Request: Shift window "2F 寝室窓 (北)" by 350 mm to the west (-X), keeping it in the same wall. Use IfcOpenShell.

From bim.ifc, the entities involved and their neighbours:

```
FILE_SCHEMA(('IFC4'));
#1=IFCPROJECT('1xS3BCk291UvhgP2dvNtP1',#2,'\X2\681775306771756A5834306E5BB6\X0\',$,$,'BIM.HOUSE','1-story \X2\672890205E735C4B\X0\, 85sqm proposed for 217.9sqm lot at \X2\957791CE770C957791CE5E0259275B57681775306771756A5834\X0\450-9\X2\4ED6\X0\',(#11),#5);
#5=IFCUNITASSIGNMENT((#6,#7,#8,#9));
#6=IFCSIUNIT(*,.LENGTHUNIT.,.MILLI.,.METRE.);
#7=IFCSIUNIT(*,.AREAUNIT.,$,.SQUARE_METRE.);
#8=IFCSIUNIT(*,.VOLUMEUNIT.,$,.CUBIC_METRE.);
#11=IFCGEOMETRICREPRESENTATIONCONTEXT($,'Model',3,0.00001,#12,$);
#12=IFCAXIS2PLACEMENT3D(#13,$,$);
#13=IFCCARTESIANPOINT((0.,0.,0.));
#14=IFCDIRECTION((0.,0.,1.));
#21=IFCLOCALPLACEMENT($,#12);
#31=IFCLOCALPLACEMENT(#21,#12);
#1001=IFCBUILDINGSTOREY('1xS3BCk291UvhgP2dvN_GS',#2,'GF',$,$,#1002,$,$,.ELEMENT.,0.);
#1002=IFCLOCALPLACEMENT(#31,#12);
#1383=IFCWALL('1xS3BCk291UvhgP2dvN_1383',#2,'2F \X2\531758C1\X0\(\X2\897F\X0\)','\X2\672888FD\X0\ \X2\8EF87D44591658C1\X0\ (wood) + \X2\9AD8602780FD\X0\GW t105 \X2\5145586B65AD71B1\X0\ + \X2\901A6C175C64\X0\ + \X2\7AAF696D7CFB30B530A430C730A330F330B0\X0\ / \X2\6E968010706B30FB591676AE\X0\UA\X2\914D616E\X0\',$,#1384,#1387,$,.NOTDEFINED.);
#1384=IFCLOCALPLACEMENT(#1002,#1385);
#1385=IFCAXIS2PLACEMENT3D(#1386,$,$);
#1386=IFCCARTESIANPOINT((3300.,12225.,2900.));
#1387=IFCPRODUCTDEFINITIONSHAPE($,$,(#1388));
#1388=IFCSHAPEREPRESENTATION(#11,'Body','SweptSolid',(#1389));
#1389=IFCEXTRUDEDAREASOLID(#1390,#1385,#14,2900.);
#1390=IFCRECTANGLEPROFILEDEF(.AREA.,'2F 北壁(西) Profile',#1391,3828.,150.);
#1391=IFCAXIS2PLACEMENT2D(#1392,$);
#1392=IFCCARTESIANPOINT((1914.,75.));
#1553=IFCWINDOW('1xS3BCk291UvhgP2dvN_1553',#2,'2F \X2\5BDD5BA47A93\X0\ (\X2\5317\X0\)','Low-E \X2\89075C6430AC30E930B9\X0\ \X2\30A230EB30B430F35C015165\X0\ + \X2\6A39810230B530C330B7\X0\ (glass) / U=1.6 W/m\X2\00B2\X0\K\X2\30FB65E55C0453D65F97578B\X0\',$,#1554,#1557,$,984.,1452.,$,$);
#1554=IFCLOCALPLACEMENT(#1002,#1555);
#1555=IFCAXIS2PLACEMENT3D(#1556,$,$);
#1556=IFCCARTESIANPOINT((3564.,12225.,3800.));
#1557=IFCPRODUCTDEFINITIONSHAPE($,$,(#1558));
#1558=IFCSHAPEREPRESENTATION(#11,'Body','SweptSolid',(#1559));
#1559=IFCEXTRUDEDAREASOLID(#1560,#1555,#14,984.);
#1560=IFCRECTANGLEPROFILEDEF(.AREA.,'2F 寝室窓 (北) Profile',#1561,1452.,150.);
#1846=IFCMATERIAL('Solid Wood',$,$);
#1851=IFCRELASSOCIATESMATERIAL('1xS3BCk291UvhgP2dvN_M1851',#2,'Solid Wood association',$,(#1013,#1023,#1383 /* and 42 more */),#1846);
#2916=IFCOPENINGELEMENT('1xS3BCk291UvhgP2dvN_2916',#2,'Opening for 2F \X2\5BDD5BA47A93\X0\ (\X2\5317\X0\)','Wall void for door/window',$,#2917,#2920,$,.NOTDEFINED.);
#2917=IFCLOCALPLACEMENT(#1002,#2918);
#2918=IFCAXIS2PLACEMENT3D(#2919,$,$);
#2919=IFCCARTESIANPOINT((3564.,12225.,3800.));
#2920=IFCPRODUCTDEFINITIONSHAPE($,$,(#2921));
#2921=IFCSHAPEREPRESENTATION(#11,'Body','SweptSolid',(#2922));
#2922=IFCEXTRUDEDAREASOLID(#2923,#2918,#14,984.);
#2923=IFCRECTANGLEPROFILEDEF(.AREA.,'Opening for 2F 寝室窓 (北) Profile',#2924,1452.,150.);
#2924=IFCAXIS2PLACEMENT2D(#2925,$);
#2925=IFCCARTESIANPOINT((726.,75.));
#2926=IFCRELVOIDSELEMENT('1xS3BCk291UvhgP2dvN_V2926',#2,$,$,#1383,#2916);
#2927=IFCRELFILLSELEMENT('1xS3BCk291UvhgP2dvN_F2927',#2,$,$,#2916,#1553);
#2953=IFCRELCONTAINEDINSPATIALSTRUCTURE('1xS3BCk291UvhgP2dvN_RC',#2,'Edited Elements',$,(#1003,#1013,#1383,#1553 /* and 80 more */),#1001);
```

```python
import ifcopenshell
import ifcopenshell.api.geometry
import ifcopenshell.util.placement
import ifcopenshell.util.unit

model = ifcopenshell.open("bim.ifc")
unit_scale = ifcopenshell.util.unit.calculate_unit_scale(model)

window = model.by_id(1553)
opening = window.FillsVoids[0].RelatingOpeningElement
wall = opening.VoidsElements[0].RelatingBuildingElement

wall_matrix = ifcopenshell.util.placement.get_local_placement(wall.ObjectPlacement)
shift = wall_matrix[:3, 0] * -0.35 / unit_scale
before = ifcopenshell.util.placement.get_local_placement(window.ObjectPlacement)[:3, 3].copy()

# The window is not placed relative to its opening, so move both.
for product in (opening, window):
    matrix = ifcopenshell.util.placement.get_local_placement(product.ObjectPlacement)
    matrix[:3, 3] += shift
    ifcopenshell.api.geometry.edit_object_placement(model, product=product, matrix=matrix, is_si=False)

after = ifcopenshell.util.placement.get_local_placement(window.ObjectPlacement)[:3, 3]
print("window moved by", (after - before).round(3) + 0.0)

model.write("bim-out.ifc")
```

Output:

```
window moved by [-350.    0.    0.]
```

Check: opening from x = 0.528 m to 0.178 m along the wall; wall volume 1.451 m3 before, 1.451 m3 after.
